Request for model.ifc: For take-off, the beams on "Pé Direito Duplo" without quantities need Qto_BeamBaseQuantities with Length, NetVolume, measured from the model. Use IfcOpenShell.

First a look at what the model holds.

```python
import ifcopenshell
import ifcopenshell.util.element
import ifcopenshell.util.unit

model = ifcopenshell.open("model.ifc")
print(model.schema)
for unit_type in ("LENGTHUNIT", "AREAUNIT", "VOLUMEUNIT"):
    print(unit_type, ifcopenshell.util.unit.calculate_unit_scale(model, unit_type))
storey = next(s for s in model.by_type("IfcBuildingStorey") if s.Name == "Pé Direito Duplo")
beams = [e for e in ifcopenshell.util.element.get_decomposition(storey) if e.is_a("IfcBeam")]
for e in sorted(beams, key=lambda e: e.id()):
    print(e.id(), e.is_a(), e.Name, list(ifcopenshell.util.element.get_psets(e, qtos_only=True)), sep=" | ")
```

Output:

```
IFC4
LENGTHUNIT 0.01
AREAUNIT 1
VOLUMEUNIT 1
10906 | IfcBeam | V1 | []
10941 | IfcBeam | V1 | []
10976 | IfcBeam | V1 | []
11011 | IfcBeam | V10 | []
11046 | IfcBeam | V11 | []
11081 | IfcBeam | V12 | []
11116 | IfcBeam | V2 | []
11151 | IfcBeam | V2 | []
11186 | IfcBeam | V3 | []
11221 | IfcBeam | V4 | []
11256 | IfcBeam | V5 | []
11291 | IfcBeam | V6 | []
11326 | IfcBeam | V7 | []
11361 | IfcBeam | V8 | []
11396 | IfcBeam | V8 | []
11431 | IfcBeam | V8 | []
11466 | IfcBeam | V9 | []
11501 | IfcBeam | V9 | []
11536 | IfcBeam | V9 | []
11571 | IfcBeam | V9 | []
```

```python
import ifcopenshell
import ifcopenshell.api.pset
import ifcopenshell.geom
import ifcopenshell.util.element
import ifcopenshell.util.shape
import ifcopenshell.util.unit

model = ifcopenshell.open("model.ifc")
unit_scale = ifcopenshell.util.unit.calculate_unit_scale(model)
volume_scale = ifcopenshell.util.unit.calculate_unit_scale(model, "VOLUMEUNIT")
settings = ifcopenshell.geom.settings()

storey = next(s for s in model.by_type("IfcBuildingStorey") if s.Name == "Pé Direito Duplo")
beams = [e for e in ifcopenshell.util.element.get_decomposition(storey) if e.is_a("IfcBeam")]

for e in sorted(beams, key=lambda e: e.id()):
    if ifcopenshell.util.element.get_psets(e, qtos_only=True, should_inherit=False):
        continue
    # Geometry comes back in metres, in the element's own axes.
    shape = ifcopenshell.geom.create_shape(settings, e)
    values = {
        "Length": ifcopenshell.util.shape.get_max_xyz(shape.geometry) / unit_scale,
        "NetVolume": ifcopenshell.util.shape.get_volume(shape.geometry) / volume_scale,
    }
    qto = ifcopenshell.api.pset.add_qto(model, product=e, name="Qto_BeamBaseQuantities")
    ifcopenshell.api.pset.edit_qto(model, qto=qto, properties=values)
    print(e.id(), {k: round(v, 3) for k, v in values.items()})

model.write("model_rev.ifc")
```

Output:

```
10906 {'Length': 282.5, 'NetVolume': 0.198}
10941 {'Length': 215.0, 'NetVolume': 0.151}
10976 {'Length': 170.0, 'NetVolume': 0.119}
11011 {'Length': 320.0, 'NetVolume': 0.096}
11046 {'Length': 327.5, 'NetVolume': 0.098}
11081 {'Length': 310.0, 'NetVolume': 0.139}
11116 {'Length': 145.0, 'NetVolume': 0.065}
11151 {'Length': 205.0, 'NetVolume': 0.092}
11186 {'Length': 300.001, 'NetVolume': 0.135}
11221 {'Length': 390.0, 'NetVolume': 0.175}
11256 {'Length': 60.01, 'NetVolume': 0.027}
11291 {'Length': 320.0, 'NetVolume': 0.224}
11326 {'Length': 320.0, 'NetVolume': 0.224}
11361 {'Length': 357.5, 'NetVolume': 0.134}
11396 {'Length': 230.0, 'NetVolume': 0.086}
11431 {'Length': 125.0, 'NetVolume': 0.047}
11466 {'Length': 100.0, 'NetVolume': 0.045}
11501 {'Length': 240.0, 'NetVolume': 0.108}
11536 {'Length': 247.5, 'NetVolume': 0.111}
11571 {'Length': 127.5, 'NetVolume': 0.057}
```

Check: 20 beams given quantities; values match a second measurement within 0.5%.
